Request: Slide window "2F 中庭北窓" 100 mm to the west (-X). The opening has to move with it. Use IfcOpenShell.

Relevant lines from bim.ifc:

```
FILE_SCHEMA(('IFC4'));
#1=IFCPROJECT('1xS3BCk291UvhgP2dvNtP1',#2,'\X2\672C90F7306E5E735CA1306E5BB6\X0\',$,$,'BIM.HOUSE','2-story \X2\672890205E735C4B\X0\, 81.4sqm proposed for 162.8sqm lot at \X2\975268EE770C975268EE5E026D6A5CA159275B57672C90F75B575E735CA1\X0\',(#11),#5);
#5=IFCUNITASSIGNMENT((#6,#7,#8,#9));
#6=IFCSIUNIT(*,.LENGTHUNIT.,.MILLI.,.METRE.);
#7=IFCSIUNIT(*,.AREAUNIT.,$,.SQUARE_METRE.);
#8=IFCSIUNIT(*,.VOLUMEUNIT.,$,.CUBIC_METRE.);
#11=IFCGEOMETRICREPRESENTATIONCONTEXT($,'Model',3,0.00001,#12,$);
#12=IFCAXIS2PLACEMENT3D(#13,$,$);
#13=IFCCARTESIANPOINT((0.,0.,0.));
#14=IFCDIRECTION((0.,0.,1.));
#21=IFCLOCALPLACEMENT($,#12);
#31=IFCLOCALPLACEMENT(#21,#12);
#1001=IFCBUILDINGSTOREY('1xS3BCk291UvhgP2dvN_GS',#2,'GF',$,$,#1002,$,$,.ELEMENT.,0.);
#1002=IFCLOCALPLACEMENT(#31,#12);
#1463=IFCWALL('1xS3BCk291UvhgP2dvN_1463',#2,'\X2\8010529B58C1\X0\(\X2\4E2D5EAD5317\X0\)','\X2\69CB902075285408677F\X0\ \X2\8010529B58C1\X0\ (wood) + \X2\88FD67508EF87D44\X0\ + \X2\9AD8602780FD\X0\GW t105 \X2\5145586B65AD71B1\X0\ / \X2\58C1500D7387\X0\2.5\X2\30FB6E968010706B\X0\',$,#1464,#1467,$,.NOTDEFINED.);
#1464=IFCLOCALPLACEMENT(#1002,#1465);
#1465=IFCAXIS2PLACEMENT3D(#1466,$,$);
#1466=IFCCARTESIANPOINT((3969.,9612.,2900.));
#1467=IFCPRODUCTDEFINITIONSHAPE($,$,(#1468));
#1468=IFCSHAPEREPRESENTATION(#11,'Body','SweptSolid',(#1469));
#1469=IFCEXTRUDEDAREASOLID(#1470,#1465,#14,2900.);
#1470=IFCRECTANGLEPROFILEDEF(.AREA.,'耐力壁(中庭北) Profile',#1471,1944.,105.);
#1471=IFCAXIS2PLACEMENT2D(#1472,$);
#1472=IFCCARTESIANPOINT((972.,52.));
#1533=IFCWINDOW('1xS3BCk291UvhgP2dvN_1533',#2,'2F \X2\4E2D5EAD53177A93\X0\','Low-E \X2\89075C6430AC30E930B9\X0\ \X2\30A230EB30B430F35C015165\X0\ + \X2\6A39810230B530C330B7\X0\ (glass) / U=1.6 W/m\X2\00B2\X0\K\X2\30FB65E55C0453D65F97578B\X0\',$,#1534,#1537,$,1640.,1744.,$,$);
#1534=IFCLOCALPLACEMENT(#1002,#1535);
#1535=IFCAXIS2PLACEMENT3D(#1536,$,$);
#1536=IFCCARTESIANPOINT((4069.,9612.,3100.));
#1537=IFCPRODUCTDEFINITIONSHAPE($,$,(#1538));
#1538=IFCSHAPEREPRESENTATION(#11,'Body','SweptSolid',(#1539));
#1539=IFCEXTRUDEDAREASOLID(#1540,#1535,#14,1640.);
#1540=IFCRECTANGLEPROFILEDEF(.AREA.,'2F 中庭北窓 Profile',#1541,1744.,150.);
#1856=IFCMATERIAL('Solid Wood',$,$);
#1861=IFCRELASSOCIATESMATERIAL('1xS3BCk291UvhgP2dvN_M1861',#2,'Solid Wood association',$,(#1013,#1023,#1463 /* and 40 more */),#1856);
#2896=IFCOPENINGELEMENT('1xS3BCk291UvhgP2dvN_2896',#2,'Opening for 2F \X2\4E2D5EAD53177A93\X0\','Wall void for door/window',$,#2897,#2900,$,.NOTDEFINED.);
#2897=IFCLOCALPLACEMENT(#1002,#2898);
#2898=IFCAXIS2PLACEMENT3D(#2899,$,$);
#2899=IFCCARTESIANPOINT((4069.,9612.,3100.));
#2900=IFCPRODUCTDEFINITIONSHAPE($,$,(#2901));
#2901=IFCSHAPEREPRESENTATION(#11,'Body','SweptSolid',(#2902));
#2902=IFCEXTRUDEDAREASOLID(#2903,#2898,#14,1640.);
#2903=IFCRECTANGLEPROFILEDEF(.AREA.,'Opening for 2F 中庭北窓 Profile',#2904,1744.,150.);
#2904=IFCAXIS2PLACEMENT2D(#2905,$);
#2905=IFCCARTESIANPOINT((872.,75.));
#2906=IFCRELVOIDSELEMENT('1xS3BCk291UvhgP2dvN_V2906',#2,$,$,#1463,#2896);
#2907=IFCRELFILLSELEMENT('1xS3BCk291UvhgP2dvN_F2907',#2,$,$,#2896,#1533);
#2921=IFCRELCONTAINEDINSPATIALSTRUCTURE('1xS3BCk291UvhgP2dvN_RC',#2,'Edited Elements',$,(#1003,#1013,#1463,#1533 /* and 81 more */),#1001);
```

```python
import ifcopenshell
import ifcopenshell.api.geometry
import ifcopenshell.util.placement
import ifcopenshell.util.unit

model = ifcopenshell.open("bim.ifc")
unit_scale = ifcopenshell.util.unit.calculate_unit_scale(model)

window = model.by_id(1533)
opening = window.FillsVoids[0].RelatingOpeningElement
wall = opening.VoidsElements[0].RelatingBuildingElement

wall_matrix = ifcopenshell.util.placement.get_local_placement(wall.ObjectPlacement)
shift = wall_matrix[:3, 0] * -0.1 / unit_scale
before = ifcopenshell.util.placement.get_local_placement(window.ObjectPlacement)[:3, 3].copy()

# The window is not placed relative to its opening, so move both.
for product in (opening, window):
    matrix = ifcopenshell.util.placement.get_local_placement(product.ObjectPlacement)
    matrix[:3, 3] += shift
    ifcopenshell.api.geometry.edit_object_placement(model, product=product, matrix=matrix, is_si=False)

after = ifcopenshell.util.placement.get_local_placement(window.ObjectPlacement)[:3, 3]
print("window moved by", (after - before).round(3) + 0.0)

model.write("bim_updated.ifc")
```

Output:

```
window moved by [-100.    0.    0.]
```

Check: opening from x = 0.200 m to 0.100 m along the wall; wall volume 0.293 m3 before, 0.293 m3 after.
